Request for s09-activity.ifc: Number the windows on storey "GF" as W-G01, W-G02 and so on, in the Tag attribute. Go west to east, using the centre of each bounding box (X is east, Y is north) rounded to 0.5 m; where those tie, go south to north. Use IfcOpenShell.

First a look at what the model holds.

```python
import ifcopenshell
import ifcopenshell.util.element
import ifcopenshell.util.placement

model = ifcopenshell.open("s09-activity.ifc")
print(model.schema)
storey = next(s for s in model.by_type("IfcBuildingStorey") if s.Name == "GF")
windows = [e for e in ifcopenshell.util.element.get_decomposition(storey) if e.is_a("IfcWindow")]
for e in sorted(windows, key=lambda e: e.id()):
    origin = ifcopenshell.util.placement.get_local_placement(e.ObjectPlacement)[:3, 3]
    print(e.id(), e.Tag, e.Name, origin.round(2) + 0.0, sep=" | ")
```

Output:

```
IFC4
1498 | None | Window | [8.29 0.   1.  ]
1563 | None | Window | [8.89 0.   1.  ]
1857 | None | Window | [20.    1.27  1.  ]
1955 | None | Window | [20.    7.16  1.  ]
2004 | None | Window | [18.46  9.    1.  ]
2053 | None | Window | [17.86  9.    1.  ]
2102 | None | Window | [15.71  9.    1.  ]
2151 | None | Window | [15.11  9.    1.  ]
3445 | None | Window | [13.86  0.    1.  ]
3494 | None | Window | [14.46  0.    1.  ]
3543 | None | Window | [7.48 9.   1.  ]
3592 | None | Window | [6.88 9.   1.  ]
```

```python
import ifcopenshell
import ifcopenshell.geom
import ifcopenshell.util.element
import ifcopenshell.util.shape

model = ifcopenshell.open("s09-activity.ifc")
settings = ifcopenshell.geom.settings()
settings.set("use-world-coords", True)


def centre(element):
    shape = ifcopenshell.geom.create_shape(settings, element)
    return ifcopenshell.util.shape.get_bbox_centroid(shape.geometry)


storey = next(s for s in model.by_type("IfcBuildingStorey") if s.Name == "GF")
windows = [e for e in ifcopenshell.util.element.get_decomposition(storey) if e.is_a("IfcWindow")]

# Insertion points can sit at a corner or the storey origin, so sort by the geometry (in metres).
centres = {e: centre(e) for e in windows}
windows.sort(key=lambda e: (round(centres[e][0] / 0.5), centres[e][1]))

for i, e in enumerate(windows, start=1):
    number = f"W-G{i:02d}"
    e.Tag = number
    print(e.id(), number)

model.write("s09-activity_v2.ifc")
```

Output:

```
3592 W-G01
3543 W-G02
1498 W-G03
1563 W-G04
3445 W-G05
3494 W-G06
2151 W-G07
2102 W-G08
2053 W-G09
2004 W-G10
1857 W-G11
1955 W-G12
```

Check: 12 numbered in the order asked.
